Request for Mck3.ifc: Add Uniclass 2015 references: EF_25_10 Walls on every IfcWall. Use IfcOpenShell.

First a look at what the model holds.

```python
import ifcopenshell

model = ifcopenshell.open("Mck3.ifc")
print(model.schema)
print("classifications:", [c.Name for c in model.by_type("IfcClassification")])
for ifc_class in ("IfcDoor", "IfcRoof", "IfcStair", "IfcWall", "IfcWindow"):
    print(ifc_class, len(model.by_type(ifc_class)))
```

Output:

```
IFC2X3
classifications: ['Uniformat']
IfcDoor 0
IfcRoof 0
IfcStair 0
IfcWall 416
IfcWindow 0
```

```python
import ifcopenshell
import ifcopenshell.api.classification

model = ifcopenshell.open("Mck3.ifc")

# IFC2X3 requires Source and Edition and has no link from the project to the system.
system = model.create_entity("IfcClassification", Source="NBS", Edition="2015", Name="Uniclass 2015")

codes = {
    "IfcWall": ("EF_25_10", "Walls"),
}
for ifc_class, (code, name) in codes.items():
    products = model.by_type(ifc_class)
    ifcopenshell.api.classification.add_reference(
        model, products=products, classification=system, identification=code, name=name
    )
    print(code, len(products))

model.write("Mck3-out.ifc")
```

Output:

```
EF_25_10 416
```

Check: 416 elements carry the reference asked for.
